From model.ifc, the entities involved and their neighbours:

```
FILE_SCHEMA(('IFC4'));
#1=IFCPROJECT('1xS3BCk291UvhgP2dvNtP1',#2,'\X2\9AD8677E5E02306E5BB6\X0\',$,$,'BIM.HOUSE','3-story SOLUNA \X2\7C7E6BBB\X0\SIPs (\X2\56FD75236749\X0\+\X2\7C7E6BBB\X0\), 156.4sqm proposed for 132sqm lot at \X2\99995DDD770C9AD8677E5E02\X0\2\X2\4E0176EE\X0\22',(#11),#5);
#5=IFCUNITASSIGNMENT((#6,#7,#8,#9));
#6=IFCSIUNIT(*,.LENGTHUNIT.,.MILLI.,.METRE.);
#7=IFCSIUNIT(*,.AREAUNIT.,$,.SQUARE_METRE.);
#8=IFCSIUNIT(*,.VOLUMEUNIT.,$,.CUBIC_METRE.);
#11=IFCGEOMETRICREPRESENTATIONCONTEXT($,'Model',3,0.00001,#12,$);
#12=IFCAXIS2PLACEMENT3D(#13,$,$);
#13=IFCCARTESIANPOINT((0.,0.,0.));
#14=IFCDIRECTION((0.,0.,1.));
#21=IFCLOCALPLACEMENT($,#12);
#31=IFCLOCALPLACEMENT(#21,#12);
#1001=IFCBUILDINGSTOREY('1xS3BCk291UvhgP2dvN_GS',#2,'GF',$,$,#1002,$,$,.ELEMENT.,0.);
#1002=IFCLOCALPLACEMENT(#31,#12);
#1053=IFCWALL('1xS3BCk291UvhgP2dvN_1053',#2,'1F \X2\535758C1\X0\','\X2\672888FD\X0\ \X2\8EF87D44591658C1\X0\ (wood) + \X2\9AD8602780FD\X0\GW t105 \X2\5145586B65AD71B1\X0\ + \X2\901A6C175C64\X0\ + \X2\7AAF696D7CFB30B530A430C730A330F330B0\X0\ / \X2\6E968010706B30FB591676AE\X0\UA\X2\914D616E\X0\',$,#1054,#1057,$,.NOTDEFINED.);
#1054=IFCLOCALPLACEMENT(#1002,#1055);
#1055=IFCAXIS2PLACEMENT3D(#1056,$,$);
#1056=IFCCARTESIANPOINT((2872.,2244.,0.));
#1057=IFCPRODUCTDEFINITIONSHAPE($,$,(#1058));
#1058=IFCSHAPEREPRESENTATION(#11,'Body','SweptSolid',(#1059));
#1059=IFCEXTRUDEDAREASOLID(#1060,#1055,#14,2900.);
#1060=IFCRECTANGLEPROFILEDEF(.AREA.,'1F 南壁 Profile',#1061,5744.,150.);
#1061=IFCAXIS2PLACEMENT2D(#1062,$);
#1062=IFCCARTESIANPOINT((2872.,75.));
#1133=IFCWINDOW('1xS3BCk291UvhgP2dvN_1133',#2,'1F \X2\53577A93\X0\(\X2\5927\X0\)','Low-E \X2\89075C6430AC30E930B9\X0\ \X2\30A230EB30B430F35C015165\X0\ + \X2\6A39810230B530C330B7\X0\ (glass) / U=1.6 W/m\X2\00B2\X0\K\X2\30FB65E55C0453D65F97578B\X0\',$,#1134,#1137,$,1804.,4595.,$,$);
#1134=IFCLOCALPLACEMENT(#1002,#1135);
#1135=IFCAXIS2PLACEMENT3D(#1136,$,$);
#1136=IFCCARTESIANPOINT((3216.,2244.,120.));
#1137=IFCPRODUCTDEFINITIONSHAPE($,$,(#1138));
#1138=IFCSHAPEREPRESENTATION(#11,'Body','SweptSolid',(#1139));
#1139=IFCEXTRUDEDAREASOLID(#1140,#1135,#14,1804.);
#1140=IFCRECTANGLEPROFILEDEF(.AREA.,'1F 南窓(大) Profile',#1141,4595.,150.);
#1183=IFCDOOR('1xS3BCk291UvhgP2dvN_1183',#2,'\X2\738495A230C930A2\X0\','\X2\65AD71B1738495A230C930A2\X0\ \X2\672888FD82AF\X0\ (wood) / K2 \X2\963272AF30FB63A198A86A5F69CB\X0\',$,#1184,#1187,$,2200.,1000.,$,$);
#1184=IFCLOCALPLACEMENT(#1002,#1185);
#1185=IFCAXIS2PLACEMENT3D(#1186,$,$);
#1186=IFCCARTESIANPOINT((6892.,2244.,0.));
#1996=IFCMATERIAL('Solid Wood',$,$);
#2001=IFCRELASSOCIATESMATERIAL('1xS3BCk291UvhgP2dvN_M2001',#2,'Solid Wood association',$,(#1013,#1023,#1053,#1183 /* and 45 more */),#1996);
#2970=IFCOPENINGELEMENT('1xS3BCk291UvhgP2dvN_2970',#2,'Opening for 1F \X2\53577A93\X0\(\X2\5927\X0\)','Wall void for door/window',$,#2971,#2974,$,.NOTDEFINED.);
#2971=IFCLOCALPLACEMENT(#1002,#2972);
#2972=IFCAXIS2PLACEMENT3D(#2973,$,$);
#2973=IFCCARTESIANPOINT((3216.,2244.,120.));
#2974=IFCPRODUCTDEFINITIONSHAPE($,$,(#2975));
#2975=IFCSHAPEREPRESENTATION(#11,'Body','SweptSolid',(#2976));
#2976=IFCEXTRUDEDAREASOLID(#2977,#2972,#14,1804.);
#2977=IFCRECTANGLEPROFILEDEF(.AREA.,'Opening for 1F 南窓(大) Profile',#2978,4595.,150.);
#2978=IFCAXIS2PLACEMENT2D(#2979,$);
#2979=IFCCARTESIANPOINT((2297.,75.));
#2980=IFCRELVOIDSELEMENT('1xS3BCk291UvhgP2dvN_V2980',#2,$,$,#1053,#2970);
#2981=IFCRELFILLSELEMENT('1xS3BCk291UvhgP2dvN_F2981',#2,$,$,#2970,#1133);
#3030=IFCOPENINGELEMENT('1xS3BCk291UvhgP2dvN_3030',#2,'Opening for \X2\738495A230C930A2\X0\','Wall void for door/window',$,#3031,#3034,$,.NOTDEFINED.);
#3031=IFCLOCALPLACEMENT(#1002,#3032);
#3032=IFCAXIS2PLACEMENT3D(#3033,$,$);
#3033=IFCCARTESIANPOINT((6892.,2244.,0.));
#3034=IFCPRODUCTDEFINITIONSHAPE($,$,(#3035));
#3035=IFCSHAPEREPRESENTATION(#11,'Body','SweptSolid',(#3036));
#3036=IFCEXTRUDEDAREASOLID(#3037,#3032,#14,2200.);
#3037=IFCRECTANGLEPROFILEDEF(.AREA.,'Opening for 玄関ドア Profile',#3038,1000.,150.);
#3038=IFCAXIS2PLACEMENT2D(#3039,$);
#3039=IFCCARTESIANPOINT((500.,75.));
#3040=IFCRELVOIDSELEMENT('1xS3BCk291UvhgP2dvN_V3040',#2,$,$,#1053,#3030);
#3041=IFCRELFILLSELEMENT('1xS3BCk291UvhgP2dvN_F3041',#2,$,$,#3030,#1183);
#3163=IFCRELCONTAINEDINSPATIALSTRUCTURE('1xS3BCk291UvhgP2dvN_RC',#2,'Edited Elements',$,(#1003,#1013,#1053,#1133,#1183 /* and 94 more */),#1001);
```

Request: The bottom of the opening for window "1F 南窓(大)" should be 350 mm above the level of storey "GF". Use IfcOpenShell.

```python
import numpy as np
import ifcopenshell
import ifcopenshell.api.geometry
import ifcopenshell.geom
import ifcopenshell.util.element
import ifcopenshell.util.placement
import ifcopenshell.util.shape
import ifcopenshell.util.unit

model = ifcopenshell.open("model.ifc")
unit_scale = ifcopenshell.util.unit.calculate_unit_scale(model)

window = model.by_id(1133)
opening = window.FillsVoids[0].RelatingOpeningElement
storey = ifcopenshell.util.element.get_container(window, ifc_class="IfcBuildingStorey")
level = ifcopenshell.util.placement.get_local_placement(storey.ObjectPlacement)[2, 3]

# The opening's origin need not be at the sill, so measure its lowest point.
shape = ifcopenshell.geom.create_shape(ifcopenshell.geom.settings(), opening)
bottom = ifcopenshell.util.shape.get_shape_bottom_elevation(shape, shape.geometry) / unit_scale
dz = level + 0.35 / unit_scale - bottom

shift = np.array([0.0, 0.0, dz])
# The window is not placed relative to its opening, so move both.
for product in (opening, window):
    matrix = ifcopenshell.util.placement.get_local_placement(product.ObjectPlacement)
    matrix[:3, 3] += shift
    ifcopenshell.api.geometry.edit_object_placement(model, product=product, matrix=matrix, is_si=False)

print(f"moved by {dz * unit_scale:+.3f} m")

model.write("model-out.ifc")
```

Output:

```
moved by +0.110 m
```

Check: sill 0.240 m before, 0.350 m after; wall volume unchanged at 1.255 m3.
